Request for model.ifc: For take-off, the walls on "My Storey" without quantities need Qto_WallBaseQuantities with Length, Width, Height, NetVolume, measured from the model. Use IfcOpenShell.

First a look at what the model holds.

```python
import ifcopenshell
import ifcopenshell.util.element
import ifcopenshell.util.unit

model = ifcopenshell.open("model.ifc")
print(model.schema)
for unit_type in ("LENGTHUNIT", "AREAUNIT", "VOLUMEUNIT"):
    print(unit_type, ifcopenshell.util.unit.calculate_unit_scale(model, unit_type))
storey = next(s for s in model.by_type("IfcBuildingStorey") if s.Name == "My Storey")
walls = [e for e in ifcopenshell.util.element.get_decomposition(storey) if e.is_a("IfcWall")]
for e in sorted(walls, key=lambda e: e.id()):
    print(e.id(), e.is_a(), e.Name, list(ifcopenshell.util.element.get_psets(e, qtos_only=True)), sep=" | ")
```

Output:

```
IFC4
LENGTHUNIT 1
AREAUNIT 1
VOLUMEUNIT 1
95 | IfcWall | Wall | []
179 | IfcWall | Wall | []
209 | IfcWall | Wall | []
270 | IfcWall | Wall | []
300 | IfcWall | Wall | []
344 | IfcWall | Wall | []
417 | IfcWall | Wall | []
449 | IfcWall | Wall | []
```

```python
import ifcopenshell
import ifcopenshell.api.pset
import ifcopenshell.geom
import ifcopenshell.util.element
import ifcopenshell.util.shape
import ifcopenshell.util.unit

model = ifcopenshell.open("model.ifc")
unit_scale = ifcopenshell.util.unit.calculate_unit_scale(model)
volume_scale = ifcopenshell.util.unit.calculate_unit_scale(model, "VOLUMEUNIT")
settings = ifcopenshell.geom.settings()

storey = next(s for s in model.by_type("IfcBuildingStorey") if s.Name == "My Storey")
walls = [e for e in ifcopenshell.util.element.get_decomposition(storey) if e.is_a("IfcWall")]

for e in sorted(walls, key=lambda e: e.id()):
    if ifcopenshell.util.element.get_psets(e, qtos_only=True, should_inherit=False):
        continue
    # Geometry comes back in metres, in the element's own axes.
    shape = ifcopenshell.geom.create_shape(settings, e)
    values = {
        "Length": ifcopenshell.util.shape.get_x(shape.geometry) / unit_scale,
        "Width": ifcopenshell.util.shape.get_y(shape.geometry) / unit_scale,
        "Height": ifcopenshell.util.shape.get_z(shape.geometry) / unit_scale,
        "NetVolume": ifcopenshell.util.shape.get_volume(shape.geometry) / volume_scale,
    }
    qto = ifcopenshell.api.pset.add_qto(model, product=e, name="Qto_WallBaseQuantities")
    ifcopenshell.api.pset.edit_qto(model, qto=qto, properties=values)
    print(e.id(), {k: round(v, 3) for k, v in values.items()})

model.write("model_updated.ifc")
```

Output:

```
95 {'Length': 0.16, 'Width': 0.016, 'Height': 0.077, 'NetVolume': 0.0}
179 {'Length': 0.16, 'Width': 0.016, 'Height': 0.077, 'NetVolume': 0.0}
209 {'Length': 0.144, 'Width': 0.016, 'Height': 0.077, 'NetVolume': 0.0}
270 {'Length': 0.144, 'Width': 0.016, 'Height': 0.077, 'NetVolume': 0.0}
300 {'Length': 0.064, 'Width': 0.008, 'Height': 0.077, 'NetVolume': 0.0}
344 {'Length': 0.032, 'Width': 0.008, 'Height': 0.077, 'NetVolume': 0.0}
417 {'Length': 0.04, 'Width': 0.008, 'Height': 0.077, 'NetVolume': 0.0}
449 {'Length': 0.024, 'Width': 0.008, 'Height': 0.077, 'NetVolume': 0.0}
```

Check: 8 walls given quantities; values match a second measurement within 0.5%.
